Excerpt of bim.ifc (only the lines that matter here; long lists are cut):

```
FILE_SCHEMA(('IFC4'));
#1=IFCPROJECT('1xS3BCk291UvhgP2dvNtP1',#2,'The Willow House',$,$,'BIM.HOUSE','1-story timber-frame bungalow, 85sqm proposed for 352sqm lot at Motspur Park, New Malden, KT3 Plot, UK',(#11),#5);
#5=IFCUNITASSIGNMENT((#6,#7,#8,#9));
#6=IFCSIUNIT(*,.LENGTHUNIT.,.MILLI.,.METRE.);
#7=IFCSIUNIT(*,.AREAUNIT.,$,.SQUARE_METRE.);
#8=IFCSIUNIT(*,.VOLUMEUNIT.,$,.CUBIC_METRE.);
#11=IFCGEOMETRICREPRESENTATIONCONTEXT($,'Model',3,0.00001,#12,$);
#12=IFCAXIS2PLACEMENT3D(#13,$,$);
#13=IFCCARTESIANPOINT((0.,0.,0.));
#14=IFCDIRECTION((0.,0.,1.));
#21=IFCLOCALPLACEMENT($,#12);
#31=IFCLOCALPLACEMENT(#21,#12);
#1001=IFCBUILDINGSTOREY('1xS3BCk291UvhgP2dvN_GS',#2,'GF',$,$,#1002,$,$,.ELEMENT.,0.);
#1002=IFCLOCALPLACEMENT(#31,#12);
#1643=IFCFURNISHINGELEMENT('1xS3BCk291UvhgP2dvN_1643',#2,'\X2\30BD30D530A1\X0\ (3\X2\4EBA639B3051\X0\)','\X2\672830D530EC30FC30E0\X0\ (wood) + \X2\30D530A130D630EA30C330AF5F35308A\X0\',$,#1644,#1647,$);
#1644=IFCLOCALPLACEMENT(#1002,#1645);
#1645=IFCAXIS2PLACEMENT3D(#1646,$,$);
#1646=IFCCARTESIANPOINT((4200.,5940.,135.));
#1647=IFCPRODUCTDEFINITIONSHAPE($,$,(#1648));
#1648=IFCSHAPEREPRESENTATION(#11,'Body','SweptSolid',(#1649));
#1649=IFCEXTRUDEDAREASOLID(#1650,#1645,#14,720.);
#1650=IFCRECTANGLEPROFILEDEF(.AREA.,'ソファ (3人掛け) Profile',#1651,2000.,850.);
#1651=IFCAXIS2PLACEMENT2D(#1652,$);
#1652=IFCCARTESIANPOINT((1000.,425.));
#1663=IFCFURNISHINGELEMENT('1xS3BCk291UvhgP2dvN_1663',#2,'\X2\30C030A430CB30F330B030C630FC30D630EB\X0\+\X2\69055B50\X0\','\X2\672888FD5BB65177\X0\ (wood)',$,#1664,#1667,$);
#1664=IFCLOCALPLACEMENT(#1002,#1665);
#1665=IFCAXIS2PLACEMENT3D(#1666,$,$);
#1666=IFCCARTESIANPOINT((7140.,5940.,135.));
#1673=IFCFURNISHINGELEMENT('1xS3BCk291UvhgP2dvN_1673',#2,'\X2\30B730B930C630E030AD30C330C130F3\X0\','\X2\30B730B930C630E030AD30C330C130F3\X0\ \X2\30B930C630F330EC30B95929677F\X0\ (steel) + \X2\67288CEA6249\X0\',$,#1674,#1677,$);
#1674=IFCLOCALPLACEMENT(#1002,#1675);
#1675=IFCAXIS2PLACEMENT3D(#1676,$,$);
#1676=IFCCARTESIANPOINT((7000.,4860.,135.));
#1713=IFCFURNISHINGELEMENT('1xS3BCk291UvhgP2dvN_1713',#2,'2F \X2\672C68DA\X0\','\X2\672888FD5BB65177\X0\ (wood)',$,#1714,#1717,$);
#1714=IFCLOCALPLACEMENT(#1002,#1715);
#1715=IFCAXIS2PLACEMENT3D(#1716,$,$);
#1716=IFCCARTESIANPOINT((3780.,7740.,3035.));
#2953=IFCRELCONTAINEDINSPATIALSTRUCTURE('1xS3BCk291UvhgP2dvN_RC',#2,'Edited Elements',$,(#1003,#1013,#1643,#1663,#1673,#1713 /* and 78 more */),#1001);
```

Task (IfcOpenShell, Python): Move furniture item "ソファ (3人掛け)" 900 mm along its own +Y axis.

```python
import ifcopenshell
import ifcopenshell.api.geometry
import ifcopenshell.util.placement
import ifcopenshell.util.unit

model = ifcopenshell.open("bim.ifc")
unit_scale = ifcopenshell.util.unit.calculate_unit_scale(model)

item = model.by_guid("1xS3BCk291UvhgP2dvN_1643")
matrix = ifcopenshell.util.placement.get_local_placement(item.ObjectPlacement)
matrix[:3, 3] += matrix[:3, 1] * 0.9 / unit_scale
ifcopenshell.api.geometry.edit_object_placement(model, product=item, matrix=matrix, is_si=False)

print(ifcopenshell.util.placement.get_local_placement(item.ObjectPlacement).round(3) + 0.0)

model.write("bim_edited.ifc")
```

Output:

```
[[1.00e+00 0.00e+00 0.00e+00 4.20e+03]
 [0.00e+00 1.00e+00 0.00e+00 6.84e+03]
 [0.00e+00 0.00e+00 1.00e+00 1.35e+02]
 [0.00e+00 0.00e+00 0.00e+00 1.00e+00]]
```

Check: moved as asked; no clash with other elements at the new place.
